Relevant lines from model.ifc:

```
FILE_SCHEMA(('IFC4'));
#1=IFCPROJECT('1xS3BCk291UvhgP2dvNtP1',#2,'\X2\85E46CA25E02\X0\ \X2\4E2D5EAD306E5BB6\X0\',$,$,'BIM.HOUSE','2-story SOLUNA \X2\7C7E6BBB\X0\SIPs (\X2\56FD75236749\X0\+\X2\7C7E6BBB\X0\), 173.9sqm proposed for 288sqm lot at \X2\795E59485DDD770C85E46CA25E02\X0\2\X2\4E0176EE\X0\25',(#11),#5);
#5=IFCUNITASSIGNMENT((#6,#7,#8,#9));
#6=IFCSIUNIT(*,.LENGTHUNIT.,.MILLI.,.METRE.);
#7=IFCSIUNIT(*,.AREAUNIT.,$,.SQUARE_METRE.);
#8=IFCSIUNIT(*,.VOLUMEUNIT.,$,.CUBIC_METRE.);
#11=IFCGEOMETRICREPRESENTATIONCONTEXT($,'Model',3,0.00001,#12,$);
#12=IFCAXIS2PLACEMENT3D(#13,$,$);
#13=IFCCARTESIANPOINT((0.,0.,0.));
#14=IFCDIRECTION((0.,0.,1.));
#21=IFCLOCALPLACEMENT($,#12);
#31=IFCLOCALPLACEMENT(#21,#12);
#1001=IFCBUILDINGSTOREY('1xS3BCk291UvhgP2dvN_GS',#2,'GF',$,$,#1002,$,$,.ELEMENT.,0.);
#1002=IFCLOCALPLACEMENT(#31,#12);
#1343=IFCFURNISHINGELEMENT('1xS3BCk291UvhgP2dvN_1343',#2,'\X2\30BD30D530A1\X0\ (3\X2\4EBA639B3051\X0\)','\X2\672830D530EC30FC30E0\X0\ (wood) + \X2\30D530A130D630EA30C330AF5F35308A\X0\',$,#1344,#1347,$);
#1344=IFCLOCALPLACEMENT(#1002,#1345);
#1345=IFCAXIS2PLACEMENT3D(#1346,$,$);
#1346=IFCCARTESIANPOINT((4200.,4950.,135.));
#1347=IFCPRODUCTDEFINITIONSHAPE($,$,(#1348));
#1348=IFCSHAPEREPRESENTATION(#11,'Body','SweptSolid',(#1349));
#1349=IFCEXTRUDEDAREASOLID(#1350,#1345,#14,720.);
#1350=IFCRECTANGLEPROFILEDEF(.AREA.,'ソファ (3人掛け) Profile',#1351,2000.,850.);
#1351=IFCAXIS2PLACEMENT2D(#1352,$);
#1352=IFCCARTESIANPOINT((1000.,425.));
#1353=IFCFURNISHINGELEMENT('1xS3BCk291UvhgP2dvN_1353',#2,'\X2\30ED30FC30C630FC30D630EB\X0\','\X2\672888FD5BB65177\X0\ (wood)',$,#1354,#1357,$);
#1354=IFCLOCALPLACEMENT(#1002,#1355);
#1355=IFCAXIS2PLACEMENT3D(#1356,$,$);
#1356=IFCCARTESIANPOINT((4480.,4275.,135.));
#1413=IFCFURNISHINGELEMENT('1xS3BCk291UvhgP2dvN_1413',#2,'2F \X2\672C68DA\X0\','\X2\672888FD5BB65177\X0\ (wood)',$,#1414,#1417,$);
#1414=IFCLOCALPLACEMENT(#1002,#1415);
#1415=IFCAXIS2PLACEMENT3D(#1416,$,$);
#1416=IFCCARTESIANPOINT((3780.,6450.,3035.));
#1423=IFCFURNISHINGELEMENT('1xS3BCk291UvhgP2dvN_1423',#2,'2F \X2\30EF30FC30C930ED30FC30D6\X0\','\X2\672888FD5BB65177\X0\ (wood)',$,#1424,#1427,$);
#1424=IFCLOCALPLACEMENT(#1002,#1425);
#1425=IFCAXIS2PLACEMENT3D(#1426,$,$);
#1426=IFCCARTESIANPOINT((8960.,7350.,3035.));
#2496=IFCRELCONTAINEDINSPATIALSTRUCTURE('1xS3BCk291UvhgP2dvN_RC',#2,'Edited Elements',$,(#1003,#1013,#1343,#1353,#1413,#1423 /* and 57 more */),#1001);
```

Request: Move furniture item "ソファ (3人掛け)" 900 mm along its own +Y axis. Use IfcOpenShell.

```python
import ifcopenshell
import ifcopenshell.api.geometry
import ifcopenshell.util.placement

model = ifcopenshell.open("model.ifc")

item = model.by_guid("1xS3BCk291UvhgP2dvN_1343")
matrix = ifcopenshell.util.placement.get_local_placement(item.ObjectPlacement)
matrix[:3, 3] += matrix[:3, 1] * 900.0
ifcopenshell.api.geometry.edit_object_placement(model, product=item, matrix=matrix, is_si=False)

print(ifcopenshell.util.placement.get_local_placement(item.ObjectPlacement).round(3) + 0.0)

model.write("model-out.ifc")
```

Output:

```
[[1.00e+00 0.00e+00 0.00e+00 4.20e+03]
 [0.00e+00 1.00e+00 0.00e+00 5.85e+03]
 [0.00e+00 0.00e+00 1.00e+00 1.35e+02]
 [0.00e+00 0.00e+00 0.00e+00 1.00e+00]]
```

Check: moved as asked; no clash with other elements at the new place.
